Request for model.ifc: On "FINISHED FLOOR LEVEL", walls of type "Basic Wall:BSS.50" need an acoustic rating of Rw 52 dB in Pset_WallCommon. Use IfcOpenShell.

First a look at what the model holds.

```python
import ifcopenshell
import ifcopenshell.util.element

model = ifcopenshell.open("model.ifc")
print(model.schema)
storey = next(s for s in model.by_type("IfcBuildingStorey") if s.Name == "FINISHED FLOOR LEVEL")
walls = [e for e in ifcopenshell.util.element.get_decomposition(storey) if e.is_a("IfcWall")]
seen = {}
for e in walls:
    element_type = ifcopenshell.util.element.get_type(e)
    key = (element_type.Name if element_type != e and element_type else None, ifcopenshell.util.element.get_pset(e, "Pset_WallCommon", "AcousticRating"))
    seen[key] = seen.get(key, 0) + 1
for (name, value), count in sorted(seen.items(), key=str):
    print(count, "x", name, "|", value)
```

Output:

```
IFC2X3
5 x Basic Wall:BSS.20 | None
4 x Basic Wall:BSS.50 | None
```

```python
import ifcopenshell
import ifcopenshell.api.pset
import ifcopenshell.util.element

model = ifcopenshell.open("model.ifc")

storey = next(s for s in model.by_type("IfcBuildingStorey") if s.Name == "FINISHED FLOOR LEVEL")
walls = [e for e in ifcopenshell.util.element.get_decomposition(storey) if e.is_a("IfcWall")]

count = 0
for e in walls:
    element_type = ifcopenshell.util.element.get_type(e)
    if element_type in (None, e) or element_type.Name != "Basic Wall:BSS.50":
        continue
    # add_pset returns the element's existing set when there is one.
    pset = ifcopenshell.api.pset.add_pset(model, product=e, name="Pset_WallCommon")
    ifcopenshell.api.pset.edit_pset(model, pset=pset, properties={"AcousticRating": "Rw 52 dB"})
    count += 1

print(count, "walls updated")

model.write("model_edited.ifc")
```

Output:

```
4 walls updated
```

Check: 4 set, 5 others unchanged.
